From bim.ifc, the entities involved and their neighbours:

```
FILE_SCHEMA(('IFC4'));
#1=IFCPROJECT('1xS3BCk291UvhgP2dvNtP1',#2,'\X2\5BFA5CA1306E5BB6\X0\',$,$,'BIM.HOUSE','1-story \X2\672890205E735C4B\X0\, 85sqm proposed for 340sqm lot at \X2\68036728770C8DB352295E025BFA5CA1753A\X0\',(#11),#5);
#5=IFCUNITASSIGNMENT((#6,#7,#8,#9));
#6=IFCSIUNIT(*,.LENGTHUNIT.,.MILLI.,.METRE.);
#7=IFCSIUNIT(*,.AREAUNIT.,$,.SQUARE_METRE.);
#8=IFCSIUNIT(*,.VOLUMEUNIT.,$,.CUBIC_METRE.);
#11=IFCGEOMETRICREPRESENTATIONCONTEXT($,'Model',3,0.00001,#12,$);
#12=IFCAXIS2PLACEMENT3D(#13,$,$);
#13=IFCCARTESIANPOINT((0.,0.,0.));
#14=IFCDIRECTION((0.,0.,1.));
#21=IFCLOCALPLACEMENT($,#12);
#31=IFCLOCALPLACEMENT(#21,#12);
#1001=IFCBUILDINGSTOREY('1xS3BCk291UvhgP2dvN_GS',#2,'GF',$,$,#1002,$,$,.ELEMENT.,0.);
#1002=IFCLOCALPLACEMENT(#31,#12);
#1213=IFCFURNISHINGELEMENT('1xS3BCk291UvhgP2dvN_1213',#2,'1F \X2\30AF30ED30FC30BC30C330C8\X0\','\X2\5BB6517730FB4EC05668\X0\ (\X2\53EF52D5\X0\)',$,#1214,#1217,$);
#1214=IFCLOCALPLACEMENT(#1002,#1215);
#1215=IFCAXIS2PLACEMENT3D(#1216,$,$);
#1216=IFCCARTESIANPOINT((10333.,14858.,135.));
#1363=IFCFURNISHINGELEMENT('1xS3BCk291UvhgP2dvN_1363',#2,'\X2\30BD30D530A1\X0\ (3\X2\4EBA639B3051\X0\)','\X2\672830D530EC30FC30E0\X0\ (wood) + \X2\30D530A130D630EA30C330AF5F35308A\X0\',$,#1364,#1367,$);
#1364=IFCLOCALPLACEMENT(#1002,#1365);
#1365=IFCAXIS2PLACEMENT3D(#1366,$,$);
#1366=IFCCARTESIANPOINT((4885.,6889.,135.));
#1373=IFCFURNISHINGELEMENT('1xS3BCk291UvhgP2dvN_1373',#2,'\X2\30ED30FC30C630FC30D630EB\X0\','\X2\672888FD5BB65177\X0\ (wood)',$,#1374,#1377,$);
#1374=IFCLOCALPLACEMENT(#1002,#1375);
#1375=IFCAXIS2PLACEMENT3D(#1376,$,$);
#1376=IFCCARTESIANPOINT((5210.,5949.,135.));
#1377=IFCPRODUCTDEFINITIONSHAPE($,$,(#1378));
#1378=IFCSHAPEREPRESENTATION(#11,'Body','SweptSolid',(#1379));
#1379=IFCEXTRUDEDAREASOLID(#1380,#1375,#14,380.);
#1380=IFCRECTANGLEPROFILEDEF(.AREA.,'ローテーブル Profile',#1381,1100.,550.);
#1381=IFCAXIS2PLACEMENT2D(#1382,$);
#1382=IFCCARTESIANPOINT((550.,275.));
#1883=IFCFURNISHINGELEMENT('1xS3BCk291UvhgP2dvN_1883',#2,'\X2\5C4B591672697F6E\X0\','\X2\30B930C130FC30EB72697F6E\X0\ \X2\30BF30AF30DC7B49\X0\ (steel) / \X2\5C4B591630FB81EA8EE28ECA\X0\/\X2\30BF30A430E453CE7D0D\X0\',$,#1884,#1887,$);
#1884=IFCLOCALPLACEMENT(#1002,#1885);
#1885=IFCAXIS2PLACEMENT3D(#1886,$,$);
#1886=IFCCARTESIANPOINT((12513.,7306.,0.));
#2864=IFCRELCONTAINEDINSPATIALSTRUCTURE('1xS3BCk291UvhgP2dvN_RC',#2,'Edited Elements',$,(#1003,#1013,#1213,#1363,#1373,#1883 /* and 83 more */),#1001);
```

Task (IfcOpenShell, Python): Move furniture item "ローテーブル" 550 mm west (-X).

```python
import ifcopenshell
import ifcopenshell.api.geometry
import ifcopenshell.util.placement
import ifcopenshell.util.unit

model = ifcopenshell.open("bim.ifc")
unit_scale = ifcopenshell.util.unit.calculate_unit_scale(model)

item = model.by_id(1373)
matrix = ifcopenshell.util.placement.get_local_placement(item.ObjectPlacement)
matrix[0, 3] -= 0.55 / unit_scale
ifcopenshell.api.geometry.edit_object_placement(model, product=item, matrix=matrix, is_si=False)

print(ifcopenshell.util.placement.get_local_placement(item.ObjectPlacement).round(3) + 0.0)

model.write("bim_edited.ifc")
```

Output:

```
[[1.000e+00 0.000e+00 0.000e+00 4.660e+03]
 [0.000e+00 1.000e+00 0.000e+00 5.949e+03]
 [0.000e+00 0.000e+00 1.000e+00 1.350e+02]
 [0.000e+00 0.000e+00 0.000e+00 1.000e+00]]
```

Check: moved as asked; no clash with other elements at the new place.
